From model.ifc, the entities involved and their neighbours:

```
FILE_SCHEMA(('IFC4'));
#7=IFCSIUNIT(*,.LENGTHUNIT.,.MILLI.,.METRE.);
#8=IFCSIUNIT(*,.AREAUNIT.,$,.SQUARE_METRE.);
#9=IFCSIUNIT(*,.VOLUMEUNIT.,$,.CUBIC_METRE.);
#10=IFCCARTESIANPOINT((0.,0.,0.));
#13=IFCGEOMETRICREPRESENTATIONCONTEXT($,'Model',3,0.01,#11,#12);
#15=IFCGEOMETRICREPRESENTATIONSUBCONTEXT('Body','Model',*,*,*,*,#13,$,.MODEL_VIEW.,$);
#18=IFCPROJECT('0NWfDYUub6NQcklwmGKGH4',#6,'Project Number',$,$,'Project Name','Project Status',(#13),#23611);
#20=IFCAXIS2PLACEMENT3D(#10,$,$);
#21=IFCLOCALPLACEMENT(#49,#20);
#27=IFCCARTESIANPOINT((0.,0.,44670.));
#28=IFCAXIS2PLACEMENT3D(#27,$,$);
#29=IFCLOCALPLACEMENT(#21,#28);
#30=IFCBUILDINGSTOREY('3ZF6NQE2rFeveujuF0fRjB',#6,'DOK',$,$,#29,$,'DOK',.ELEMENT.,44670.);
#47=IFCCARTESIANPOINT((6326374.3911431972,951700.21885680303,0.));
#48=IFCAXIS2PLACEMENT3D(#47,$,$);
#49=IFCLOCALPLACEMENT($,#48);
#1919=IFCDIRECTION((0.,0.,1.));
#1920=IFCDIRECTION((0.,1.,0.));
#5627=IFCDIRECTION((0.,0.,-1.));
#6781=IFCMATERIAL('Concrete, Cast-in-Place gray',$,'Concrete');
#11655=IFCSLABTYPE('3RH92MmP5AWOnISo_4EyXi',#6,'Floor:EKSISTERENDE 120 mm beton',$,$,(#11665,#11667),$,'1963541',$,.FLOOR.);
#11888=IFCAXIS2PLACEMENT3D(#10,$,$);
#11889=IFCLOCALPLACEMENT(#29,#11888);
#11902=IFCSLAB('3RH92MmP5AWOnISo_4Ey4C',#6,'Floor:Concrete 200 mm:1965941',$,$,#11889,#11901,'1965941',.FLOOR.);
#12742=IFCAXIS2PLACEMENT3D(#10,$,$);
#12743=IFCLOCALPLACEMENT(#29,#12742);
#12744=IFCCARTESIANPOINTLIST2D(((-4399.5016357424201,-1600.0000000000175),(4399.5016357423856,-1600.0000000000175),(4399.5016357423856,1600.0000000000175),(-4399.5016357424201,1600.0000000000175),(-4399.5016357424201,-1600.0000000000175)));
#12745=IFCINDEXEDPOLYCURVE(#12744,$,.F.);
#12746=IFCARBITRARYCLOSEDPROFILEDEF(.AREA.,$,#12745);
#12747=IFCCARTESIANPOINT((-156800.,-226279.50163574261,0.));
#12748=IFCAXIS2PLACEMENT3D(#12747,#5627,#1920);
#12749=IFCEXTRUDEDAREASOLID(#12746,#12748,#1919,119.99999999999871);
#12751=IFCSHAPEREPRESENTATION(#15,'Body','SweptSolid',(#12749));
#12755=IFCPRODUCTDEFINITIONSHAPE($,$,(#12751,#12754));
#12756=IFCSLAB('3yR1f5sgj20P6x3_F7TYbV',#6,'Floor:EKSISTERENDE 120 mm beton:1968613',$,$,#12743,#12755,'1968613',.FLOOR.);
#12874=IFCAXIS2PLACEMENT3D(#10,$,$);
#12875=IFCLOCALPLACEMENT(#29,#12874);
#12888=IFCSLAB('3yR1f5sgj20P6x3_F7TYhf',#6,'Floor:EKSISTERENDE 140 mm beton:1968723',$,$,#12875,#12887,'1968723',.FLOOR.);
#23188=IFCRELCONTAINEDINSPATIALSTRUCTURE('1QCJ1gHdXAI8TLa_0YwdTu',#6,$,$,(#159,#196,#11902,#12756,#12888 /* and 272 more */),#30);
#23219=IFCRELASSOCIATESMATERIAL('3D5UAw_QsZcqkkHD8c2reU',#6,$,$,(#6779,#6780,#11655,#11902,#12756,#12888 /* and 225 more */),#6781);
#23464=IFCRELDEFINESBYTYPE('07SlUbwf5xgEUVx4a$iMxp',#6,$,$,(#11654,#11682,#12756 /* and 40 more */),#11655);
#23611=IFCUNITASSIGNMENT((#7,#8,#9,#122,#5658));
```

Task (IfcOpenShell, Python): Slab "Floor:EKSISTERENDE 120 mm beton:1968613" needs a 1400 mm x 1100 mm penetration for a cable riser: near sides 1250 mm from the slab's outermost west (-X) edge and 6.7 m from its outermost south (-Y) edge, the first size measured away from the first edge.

```python
import numpy as np
import ifcopenshell
import ifcopenshell.api.feature
import ifcopenshell.api.geometry
import ifcopenshell.api.root
import ifcopenshell.geom
import ifcopenshell.util.placement
import ifcopenshell.util.representation
import ifcopenshell.util.shape
import ifcopenshell.util.unit

model = ifcopenshell.open("model.ifc")
unit_scale = ifcopenshell.util.unit.calculate_unit_scale(model)
settings = ifcopenshell.geom.settings()


def volume(element):
    """Net volume in cubic metres, openings subtracted."""
    shape = ifcopenshell.geom.create_shape(settings, element)
    return ifcopenshell.util.shape.get_volume(shape.geometry)


slab = model.by_guid("3yR1f5sgj20P6x3_F7TYbV")
before = volume(slab)

# Extent in the slab's own axes, in metres. The edges named are its -X and -Y sides.
slab_shape = ifcopenshell.geom.create_shape(settings, slab)
vertices = ifcopenshell.util.shape.get_vertices(slab_shape.geometry)
x_min, y_min, bottom = vertices.min(axis=0)
top = vertices[:, 2].max()

opening = ifcopenshell.api.root.create_entity(model, ifc_class="IfcOpeningElement", name="Cable riser opening", predefined_type="OPENING")
context = ifcopenshell.util.representation.get_context(model, "Model", "Body", "MODEL_VIEW")
width, depth = 1.4, 1.1
outline = [(0.0, 0.0), (width, 0.0), (width, depth), (0.0, depth), (0.0, 0.0)]
# Overshoot both faces by 50 mm so the cut is clean.
shape = ifcopenshell.api.geometry.add_slab_representation(
    model, context=context, depth=top - bottom + 0.1, polyline=outline
)
ifcopenshell.api.geometry.assign_representation(model, product=opening, representation=shape)

matrix = ifcopenshell.util.placement.get_local_placement(slab.ObjectPlacement)
matrix[:, 3] = matrix @ np.append(np.array([x_min + 1.25, y_min + 6.7, bottom - 0.05]) / unit_scale, 1.0)
ifcopenshell.api.geometry.edit_object_placement(model, product=opening, matrix=matrix, is_si=False)
ifcopenshell.api.feature.add_feature(model, feature=opening, element=slab)

after = volume(slab)

print(f"slab volume {before:.3f} -> {after:.3f} m3")

model.write("model_edited.ifc")
```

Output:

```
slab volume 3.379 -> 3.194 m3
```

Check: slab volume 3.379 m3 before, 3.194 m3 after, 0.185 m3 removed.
